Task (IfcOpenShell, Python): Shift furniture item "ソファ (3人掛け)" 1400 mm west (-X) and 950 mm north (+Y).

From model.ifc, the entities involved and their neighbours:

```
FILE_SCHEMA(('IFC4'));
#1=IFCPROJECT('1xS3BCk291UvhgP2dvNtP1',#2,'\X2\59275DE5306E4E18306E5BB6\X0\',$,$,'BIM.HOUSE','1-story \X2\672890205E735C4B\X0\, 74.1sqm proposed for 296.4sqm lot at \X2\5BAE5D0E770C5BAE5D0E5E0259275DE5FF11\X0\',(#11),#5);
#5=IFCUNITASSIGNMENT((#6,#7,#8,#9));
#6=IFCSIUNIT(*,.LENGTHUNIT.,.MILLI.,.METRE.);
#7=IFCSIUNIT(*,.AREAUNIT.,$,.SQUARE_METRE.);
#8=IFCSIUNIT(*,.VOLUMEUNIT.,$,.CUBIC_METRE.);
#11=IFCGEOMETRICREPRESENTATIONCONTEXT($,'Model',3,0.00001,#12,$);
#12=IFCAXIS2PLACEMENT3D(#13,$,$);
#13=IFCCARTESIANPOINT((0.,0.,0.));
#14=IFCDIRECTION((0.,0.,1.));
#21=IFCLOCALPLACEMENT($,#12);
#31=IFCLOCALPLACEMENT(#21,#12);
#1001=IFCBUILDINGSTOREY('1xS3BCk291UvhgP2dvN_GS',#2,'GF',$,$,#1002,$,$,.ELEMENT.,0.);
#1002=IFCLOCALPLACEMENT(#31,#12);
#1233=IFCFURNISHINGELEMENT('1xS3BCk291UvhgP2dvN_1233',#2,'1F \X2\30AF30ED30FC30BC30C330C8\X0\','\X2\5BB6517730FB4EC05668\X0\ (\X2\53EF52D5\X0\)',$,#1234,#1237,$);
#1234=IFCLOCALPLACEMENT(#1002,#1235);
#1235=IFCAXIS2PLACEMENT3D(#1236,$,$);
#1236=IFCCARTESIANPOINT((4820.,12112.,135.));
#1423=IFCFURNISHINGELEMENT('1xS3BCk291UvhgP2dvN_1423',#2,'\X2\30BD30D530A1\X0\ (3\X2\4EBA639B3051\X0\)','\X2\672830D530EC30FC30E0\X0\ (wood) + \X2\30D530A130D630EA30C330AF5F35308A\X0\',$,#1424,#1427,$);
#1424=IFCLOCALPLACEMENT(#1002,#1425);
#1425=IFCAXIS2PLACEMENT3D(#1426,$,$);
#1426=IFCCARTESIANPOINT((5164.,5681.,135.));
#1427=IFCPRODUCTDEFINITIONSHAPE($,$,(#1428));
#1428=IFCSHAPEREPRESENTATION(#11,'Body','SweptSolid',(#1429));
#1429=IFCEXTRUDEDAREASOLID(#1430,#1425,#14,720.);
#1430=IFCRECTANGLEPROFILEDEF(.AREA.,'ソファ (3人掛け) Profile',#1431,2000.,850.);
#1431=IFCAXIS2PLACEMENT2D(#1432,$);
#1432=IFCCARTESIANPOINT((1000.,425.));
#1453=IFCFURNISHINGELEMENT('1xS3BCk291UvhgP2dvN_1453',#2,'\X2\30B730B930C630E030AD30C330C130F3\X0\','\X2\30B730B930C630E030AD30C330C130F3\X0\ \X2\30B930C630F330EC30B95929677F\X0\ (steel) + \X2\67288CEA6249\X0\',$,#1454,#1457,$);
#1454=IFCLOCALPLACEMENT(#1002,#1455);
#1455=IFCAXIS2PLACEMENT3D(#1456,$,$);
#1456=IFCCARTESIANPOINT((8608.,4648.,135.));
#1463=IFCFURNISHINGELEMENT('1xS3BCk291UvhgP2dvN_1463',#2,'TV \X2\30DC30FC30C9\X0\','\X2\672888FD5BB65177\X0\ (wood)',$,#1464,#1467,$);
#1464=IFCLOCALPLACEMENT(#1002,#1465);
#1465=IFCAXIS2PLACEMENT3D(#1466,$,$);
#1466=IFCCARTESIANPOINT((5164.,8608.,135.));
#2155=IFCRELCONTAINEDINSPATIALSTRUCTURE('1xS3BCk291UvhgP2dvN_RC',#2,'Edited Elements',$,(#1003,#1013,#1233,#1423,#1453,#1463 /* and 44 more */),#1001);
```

```python
import ifcopenshell
import ifcopenshell.api.geometry
import ifcopenshell.util.placement

model = ifcopenshell.open("model.ifc")

item = model.by_guid("1xS3BCk291UvhgP2dvN_1423")
matrix = ifcopenshell.util.placement.get_local_placement(item.ObjectPlacement)
matrix[0, 3] -= 1400.0
matrix[1, 3] += 950.0
ifcopenshell.api.geometry.edit_object_placement(model, product=item, matrix=matrix, is_si=False)

print(ifcopenshell.util.placement.get_local_placement(item.ObjectPlacement).round(3) + 0.0)

model.write("model_v2.ifc")
```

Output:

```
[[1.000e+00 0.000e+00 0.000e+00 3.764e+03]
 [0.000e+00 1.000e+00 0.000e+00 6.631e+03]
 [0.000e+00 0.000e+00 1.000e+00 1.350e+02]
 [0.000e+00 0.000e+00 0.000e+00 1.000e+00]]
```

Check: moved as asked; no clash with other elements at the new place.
